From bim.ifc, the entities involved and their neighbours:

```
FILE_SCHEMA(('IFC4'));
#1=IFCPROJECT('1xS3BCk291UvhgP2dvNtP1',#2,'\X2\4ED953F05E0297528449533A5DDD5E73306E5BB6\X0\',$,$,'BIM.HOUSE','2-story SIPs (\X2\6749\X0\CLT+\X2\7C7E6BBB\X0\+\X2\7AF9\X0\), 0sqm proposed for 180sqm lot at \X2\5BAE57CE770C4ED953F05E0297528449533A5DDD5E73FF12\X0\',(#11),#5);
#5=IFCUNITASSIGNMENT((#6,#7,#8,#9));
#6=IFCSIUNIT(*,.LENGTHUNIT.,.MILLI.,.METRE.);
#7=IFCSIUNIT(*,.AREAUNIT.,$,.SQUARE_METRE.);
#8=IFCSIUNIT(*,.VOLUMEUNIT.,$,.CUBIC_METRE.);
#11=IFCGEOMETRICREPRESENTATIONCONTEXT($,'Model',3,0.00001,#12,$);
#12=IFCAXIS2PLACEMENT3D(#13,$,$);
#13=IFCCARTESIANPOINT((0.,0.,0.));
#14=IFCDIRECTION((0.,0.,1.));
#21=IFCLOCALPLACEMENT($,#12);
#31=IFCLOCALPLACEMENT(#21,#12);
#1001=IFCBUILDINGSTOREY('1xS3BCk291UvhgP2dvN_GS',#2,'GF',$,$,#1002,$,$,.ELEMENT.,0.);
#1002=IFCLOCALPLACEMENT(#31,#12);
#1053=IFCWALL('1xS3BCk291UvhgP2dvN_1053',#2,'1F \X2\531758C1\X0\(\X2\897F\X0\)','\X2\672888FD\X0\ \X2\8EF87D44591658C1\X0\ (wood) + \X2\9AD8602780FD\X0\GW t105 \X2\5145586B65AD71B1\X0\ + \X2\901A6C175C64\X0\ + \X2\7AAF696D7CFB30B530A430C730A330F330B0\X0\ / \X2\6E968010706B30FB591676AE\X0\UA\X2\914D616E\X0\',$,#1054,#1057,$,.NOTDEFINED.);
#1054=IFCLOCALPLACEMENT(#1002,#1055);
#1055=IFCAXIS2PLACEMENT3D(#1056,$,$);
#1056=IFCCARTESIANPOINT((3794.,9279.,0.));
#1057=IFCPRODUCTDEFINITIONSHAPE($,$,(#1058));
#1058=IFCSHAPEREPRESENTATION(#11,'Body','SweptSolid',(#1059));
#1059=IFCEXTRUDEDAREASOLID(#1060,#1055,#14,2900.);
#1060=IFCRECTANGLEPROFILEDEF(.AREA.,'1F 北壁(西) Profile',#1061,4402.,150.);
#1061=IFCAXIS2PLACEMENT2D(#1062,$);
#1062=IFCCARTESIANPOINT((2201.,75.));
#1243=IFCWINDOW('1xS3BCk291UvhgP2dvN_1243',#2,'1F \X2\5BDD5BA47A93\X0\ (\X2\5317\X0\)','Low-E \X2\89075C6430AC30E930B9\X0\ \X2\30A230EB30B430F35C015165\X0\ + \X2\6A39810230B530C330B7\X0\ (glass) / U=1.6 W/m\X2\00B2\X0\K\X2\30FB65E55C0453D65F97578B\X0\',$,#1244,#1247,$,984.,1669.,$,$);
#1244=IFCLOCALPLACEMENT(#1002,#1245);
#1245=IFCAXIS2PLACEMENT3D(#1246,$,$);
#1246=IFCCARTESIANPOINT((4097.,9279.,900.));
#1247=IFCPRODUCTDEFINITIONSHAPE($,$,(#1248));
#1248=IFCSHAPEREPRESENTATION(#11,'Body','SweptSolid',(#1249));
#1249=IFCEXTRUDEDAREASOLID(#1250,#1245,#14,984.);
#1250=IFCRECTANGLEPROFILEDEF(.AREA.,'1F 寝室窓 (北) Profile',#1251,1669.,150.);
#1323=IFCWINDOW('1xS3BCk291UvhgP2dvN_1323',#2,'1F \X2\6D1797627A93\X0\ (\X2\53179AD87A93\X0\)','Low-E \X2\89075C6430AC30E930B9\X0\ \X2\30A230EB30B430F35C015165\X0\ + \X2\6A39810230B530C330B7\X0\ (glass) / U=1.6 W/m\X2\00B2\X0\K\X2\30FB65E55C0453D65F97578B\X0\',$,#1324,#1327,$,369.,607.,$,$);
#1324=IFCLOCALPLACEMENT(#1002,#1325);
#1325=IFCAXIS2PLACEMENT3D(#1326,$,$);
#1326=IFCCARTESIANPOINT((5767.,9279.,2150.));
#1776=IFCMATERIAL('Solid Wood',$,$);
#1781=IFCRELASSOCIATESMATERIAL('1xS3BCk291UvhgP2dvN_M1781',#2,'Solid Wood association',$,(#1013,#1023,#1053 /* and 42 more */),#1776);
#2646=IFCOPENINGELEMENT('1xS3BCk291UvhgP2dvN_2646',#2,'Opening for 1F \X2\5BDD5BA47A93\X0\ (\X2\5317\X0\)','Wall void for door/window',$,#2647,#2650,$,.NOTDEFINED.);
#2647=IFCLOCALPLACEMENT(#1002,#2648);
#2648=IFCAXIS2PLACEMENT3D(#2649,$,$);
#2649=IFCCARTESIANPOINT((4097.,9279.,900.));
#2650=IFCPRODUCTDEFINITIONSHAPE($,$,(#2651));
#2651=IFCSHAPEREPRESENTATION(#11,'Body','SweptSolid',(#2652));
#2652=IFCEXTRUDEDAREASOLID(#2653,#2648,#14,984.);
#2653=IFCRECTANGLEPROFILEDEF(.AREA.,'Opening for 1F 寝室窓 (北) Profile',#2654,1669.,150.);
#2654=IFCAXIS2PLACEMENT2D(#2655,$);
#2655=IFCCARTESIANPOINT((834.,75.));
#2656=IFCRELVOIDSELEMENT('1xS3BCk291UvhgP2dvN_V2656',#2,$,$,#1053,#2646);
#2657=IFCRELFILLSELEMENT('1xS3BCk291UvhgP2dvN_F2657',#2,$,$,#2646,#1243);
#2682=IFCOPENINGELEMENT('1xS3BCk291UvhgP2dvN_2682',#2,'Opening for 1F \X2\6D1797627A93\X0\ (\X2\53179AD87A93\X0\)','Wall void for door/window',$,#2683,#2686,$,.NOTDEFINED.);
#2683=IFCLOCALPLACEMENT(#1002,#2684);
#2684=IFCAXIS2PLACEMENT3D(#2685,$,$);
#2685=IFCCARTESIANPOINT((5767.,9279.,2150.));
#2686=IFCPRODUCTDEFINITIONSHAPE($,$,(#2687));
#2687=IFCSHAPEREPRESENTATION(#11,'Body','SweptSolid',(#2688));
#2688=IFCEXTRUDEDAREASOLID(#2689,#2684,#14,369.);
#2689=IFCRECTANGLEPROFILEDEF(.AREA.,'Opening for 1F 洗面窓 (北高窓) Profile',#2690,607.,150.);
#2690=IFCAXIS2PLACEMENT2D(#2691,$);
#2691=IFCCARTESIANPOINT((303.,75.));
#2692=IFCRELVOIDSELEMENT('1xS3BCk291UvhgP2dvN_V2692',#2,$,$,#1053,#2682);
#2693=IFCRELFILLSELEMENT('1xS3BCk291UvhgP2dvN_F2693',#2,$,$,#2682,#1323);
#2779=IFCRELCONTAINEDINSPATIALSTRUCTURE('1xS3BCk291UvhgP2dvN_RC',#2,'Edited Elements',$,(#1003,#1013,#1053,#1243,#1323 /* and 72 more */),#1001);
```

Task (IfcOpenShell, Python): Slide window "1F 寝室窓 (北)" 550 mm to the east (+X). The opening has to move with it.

```python
import ifcopenshell
import ifcopenshell.api.geometry
import ifcopenshell.util.placement
import ifcopenshell.util.unit

model = ifcopenshell.open("bim.ifc")
unit_scale = ifcopenshell.util.unit.calculate_unit_scale(model)

window = model.by_id(1243)
opening = window.FillsVoids[0].RelatingOpeningElement
wall = opening.VoidsElements[0].RelatingBuildingElement

wall_matrix = ifcopenshell.util.placement.get_local_placement(wall.ObjectPlacement)
shift = wall_matrix[:3, 0] * 0.55 / unit_scale
before = ifcopenshell.util.placement.get_local_placement(window.ObjectPlacement)[:3, 3].copy()

# The window is not placed relative to its opening, so move both.
for product in (opening, window):
    matrix = ifcopenshell.util.placement.get_local_placement(product.ObjectPlacement)
    matrix[:3, 3] += shift
    ifcopenshell.api.geometry.edit_object_placement(model, product=product, matrix=matrix, is_si=False)

after = ifcopenshell.util.placement.get_local_placement(window.ObjectPlacement)[:3, 3]
print("window moved by", (after - before).round(3) + 0.0)

model.write("bim_rev.ifc")
```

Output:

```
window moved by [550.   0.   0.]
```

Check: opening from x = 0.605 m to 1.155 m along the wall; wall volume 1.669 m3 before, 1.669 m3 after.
